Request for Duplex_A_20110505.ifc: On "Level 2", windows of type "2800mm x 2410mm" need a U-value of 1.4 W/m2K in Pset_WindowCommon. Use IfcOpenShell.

First a look at what the model holds.

```python
import ifcopenshell
import ifcopenshell.util.element

model = ifcopenshell.open("Duplex_A_20110505.ifc")
print(model.schema)
storey = next(s for s in model.by_type("IfcBuildingStorey") if s.Name == "Level 2")
windows = [e for e in ifcopenshell.util.element.get_decomposition(storey) if e.is_a("IfcWindow")]
seen = {}
for e in windows:
    element_type = ifcopenshell.util.element.get_type(e)
    key = (element_type.Name if element_type != e and element_type else None, ifcopenshell.util.element.get_pset(e, "Pset_WindowCommon", "ThermalTransmittance"))
    seen[key] = seen.get(key, 0) + 1
for (name, value), count in sorted(seen.items(), key=str):
    print(count, "x", name, "|", value)
```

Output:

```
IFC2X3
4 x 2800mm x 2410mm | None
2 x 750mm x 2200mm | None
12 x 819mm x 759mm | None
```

```python
import ifcopenshell
import ifcopenshell.api.pset
import ifcopenshell.util.element

model = ifcopenshell.open("Duplex_A_20110505.ifc")

storey = next(s for s in model.by_type("IfcBuildingStorey") if s.Name == "Level 2")
windows = [e for e in ifcopenshell.util.element.get_decomposition(storey) if e.is_a("IfcWindow")]

count = 0
for e in windows:
    element_type = ifcopenshell.util.element.get_type(e)
    if element_type in (None, e) or element_type.Name != "2800mm x 2410mm":
        continue
    # add_pset returns the element's existing set when there is one.
    pset = ifcopenshell.api.pset.add_pset(model, product=e, name="Pset_WindowCommon")
    ifcopenshell.api.pset.edit_pset(model, pset=pset, properties={"ThermalTransmittance": 1.4})
    count += 1

print(count, "windows updated")

model.write("Duplex_A_20110505_rev.ifc")
```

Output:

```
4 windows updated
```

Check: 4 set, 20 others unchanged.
